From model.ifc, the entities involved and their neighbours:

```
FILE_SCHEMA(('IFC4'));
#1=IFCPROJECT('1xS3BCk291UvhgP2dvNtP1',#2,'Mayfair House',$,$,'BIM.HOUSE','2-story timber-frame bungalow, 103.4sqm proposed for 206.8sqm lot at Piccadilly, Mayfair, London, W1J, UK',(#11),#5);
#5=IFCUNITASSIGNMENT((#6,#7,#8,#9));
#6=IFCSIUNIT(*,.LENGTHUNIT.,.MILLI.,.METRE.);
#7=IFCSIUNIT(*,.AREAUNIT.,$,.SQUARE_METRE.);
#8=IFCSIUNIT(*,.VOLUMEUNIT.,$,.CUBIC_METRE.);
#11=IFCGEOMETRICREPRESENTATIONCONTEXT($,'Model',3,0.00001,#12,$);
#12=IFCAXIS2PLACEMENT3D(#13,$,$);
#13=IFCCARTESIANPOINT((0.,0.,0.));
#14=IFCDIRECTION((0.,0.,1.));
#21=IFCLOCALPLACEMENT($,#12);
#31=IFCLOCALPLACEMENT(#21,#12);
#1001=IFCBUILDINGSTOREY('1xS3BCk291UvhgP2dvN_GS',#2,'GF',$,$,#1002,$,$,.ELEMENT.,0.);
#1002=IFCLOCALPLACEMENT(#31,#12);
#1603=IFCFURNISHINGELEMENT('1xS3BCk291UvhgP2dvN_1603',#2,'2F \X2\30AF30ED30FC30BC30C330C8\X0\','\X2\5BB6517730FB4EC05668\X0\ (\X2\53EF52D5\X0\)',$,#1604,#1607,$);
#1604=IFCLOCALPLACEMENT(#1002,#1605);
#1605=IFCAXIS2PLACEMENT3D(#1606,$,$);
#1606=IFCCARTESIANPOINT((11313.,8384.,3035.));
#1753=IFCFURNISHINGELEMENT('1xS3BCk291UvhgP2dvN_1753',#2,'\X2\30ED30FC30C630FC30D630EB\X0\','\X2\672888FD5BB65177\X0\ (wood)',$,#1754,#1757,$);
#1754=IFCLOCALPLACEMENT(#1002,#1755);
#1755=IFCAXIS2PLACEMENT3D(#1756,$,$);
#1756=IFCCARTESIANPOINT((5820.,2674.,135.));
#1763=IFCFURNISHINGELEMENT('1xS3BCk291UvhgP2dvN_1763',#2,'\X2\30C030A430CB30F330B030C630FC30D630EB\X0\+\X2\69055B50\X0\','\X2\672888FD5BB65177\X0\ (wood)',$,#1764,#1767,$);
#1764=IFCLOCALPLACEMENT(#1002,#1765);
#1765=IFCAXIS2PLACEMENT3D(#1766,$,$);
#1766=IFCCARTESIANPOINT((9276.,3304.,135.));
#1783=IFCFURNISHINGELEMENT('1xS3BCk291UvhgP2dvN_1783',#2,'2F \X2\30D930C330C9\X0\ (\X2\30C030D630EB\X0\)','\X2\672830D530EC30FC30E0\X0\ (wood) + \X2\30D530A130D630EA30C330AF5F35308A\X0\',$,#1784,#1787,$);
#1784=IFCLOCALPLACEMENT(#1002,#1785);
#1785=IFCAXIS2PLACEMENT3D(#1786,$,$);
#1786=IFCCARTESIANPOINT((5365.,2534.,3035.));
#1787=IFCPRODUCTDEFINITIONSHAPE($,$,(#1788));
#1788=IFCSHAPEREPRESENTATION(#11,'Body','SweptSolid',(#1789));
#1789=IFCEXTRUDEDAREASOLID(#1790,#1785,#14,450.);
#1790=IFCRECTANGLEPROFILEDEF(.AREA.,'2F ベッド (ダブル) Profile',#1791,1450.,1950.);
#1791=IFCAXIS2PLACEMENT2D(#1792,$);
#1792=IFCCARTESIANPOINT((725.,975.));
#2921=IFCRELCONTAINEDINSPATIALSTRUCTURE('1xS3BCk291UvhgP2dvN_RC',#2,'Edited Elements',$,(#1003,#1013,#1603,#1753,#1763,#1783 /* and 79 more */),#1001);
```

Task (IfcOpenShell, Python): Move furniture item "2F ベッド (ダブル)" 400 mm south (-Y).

```python
import ifcopenshell
import ifcopenshell.api.geometry
import ifcopenshell.util.placement

model = ifcopenshell.open("model.ifc")

item = model.by_id(1783)
matrix = ifcopenshell.util.placement.get_local_placement(item.ObjectPlacement)
matrix[1, 3] -= 400.0
ifcopenshell.api.geometry.edit_object_placement(model, product=item, matrix=matrix, is_si=False)

print(ifcopenshell.util.placement.get_local_placement(item.ObjectPlacement).round(3) + 0.0)

model.write("model_updated.ifc")
```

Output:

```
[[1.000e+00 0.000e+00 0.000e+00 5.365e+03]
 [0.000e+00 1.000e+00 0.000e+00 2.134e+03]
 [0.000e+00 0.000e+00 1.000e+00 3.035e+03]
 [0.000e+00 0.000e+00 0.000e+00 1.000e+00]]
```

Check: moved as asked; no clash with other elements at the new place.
